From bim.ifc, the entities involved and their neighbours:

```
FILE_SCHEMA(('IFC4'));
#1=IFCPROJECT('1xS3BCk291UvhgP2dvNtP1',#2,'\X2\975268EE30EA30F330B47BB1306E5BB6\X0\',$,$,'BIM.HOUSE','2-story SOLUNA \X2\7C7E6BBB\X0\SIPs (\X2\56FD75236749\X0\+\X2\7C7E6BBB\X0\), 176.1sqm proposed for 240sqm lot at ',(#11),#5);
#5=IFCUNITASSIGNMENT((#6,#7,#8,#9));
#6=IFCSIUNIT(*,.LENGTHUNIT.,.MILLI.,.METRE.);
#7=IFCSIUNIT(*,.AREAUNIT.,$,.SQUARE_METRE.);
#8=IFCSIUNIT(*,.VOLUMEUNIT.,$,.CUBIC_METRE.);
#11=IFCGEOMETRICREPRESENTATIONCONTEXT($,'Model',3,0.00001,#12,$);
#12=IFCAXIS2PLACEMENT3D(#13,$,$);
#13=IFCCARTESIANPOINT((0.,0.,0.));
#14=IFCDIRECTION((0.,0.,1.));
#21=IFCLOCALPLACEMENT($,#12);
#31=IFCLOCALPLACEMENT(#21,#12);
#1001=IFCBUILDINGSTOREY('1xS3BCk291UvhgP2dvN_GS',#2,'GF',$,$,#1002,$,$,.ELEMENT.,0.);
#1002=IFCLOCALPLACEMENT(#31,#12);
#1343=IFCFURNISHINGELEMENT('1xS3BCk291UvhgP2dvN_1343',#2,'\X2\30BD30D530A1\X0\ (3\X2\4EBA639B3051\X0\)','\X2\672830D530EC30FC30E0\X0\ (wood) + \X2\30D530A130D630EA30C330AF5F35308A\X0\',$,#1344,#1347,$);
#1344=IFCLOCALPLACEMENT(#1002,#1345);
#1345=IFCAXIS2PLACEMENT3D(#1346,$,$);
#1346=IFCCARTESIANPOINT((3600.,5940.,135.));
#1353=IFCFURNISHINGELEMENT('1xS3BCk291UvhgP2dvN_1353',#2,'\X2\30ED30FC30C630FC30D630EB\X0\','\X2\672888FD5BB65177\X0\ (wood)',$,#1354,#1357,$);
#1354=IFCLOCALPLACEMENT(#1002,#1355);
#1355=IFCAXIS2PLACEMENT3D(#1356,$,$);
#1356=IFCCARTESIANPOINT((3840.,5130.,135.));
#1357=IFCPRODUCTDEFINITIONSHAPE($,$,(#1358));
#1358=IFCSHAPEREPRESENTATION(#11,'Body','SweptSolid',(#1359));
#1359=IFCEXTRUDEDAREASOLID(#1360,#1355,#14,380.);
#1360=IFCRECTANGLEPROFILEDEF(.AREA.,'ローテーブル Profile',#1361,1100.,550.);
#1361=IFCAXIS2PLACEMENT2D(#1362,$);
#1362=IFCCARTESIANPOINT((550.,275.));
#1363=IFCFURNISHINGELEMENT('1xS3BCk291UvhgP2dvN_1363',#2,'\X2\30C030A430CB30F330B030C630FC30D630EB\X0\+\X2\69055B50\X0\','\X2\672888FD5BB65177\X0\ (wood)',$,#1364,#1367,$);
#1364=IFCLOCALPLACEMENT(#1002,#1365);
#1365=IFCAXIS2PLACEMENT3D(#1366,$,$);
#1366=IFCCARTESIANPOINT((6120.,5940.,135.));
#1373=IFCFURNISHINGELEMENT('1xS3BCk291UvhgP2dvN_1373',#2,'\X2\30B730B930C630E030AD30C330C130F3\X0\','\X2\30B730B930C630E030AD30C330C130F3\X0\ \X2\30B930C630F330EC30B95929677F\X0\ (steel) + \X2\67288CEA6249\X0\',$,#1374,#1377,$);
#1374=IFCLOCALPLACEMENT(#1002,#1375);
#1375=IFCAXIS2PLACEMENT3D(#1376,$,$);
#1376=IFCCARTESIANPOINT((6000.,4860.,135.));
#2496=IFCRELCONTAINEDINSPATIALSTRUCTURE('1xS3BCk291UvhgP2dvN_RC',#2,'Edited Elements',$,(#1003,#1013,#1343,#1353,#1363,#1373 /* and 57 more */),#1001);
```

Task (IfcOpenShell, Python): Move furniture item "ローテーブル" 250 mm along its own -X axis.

```python
import ifcopenshell
import ifcopenshell.api.geometry
import ifcopenshell.util.placement

model = ifcopenshell.open("bim.ifc")

item = model.by_guid("1xS3BCk291UvhgP2dvN_1353")
matrix = ifcopenshell.util.placement.get_local_placement(item.ObjectPlacement)
matrix[:3, 3] -= matrix[:3, 0] * 250.0
ifcopenshell.api.geometry.edit_object_placement(model, product=item, matrix=matrix, is_si=False)

print(ifcopenshell.util.placement.get_local_placement(item.ObjectPlacement).round(3) + 0.0)

model.write("bim-out.ifc")
```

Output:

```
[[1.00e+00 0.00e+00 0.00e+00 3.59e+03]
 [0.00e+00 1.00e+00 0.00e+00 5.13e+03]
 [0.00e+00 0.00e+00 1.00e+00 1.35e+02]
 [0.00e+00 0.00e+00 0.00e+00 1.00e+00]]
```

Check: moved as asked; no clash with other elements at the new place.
